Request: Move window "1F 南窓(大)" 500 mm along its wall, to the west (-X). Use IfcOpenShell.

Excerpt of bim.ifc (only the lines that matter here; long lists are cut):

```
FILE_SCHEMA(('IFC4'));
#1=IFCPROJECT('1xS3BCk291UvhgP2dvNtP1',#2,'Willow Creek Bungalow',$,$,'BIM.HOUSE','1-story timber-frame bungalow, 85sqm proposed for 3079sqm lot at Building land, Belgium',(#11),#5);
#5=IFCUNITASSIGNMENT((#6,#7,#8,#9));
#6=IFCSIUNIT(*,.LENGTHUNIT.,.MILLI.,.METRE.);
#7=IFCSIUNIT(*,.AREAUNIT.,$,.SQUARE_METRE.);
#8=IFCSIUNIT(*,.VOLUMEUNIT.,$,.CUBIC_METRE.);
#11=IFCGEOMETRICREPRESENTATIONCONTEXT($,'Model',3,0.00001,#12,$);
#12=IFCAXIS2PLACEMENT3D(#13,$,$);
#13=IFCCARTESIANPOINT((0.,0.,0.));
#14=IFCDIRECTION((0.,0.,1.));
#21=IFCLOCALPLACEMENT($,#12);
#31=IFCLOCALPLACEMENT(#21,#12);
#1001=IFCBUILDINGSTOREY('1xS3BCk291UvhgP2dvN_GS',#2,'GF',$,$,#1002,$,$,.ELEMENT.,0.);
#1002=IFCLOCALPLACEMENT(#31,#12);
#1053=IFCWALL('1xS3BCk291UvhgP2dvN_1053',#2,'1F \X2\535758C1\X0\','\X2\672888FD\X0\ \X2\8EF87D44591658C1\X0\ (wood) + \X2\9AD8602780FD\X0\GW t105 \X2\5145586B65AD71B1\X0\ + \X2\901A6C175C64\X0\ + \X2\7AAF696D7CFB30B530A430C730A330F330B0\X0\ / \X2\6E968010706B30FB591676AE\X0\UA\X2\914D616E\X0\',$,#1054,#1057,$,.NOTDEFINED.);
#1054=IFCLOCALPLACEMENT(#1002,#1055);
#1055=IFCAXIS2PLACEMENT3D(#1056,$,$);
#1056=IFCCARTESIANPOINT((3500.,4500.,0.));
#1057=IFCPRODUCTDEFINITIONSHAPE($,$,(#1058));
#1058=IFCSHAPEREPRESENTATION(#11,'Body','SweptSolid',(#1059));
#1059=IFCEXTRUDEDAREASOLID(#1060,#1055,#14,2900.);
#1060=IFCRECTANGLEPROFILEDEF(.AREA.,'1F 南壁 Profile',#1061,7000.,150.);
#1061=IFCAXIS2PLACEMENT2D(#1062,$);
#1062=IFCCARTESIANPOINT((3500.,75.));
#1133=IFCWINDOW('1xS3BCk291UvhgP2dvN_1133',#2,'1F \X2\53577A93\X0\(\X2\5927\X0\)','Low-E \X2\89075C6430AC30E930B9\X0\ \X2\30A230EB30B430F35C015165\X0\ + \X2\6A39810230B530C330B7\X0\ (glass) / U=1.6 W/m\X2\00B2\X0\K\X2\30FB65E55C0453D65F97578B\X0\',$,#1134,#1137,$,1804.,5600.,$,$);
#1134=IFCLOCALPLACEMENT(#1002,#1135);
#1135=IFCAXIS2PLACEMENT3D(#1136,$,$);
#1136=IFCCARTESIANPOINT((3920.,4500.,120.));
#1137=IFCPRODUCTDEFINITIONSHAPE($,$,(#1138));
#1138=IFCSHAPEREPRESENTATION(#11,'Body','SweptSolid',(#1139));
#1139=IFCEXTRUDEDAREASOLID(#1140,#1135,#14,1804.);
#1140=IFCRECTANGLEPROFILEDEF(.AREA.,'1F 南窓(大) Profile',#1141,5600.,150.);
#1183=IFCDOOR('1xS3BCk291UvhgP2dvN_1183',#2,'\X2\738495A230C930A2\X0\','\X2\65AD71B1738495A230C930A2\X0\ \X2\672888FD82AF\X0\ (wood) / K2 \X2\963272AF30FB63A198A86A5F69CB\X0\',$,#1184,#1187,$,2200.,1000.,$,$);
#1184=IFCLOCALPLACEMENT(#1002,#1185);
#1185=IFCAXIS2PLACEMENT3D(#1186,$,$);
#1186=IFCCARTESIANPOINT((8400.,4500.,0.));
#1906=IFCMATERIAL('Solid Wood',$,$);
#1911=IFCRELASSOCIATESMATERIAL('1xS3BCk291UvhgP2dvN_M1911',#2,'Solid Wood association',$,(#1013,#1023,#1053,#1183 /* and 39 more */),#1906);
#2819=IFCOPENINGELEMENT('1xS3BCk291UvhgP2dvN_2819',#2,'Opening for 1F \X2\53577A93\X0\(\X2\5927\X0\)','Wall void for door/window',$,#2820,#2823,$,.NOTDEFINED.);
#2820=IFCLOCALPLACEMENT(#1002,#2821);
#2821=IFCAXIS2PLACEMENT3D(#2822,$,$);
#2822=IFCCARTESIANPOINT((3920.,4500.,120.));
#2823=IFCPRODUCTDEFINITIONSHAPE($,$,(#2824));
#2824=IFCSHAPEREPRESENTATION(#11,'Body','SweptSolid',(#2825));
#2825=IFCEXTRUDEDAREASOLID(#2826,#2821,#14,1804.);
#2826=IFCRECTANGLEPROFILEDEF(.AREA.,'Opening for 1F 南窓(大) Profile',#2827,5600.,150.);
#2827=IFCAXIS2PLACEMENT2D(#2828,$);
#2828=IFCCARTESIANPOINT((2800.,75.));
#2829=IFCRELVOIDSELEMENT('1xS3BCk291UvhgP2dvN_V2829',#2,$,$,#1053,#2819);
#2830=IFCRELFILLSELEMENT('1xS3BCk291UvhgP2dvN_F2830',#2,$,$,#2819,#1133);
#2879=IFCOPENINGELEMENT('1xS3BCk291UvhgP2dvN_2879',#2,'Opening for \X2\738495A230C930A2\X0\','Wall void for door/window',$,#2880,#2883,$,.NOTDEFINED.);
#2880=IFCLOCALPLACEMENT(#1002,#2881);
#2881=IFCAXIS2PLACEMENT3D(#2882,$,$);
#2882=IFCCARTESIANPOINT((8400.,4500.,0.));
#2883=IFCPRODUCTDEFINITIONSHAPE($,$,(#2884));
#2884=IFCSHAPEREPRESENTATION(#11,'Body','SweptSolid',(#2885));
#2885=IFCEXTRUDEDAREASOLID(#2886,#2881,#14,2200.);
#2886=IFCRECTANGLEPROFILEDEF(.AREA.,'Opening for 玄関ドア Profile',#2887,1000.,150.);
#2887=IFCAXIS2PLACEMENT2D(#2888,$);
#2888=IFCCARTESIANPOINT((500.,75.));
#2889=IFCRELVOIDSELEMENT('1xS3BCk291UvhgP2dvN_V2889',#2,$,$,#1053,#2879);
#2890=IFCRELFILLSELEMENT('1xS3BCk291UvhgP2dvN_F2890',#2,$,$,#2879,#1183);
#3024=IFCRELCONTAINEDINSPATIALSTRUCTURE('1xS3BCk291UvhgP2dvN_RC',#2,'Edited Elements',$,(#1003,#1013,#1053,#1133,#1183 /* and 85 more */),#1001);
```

```python
import ifcopenshell
import ifcopenshell.api.geometry
import ifcopenshell.util.placement

model = ifcopenshell.open("bim.ifc")

window = model.by_guid("1xS3BCk291UvhgP2dvN_1133")
opening = window.FillsVoids[0].RelatingOpeningElement
wall = opening.VoidsElements[0].RelatingBuildingElement

wall_matrix = ifcopenshell.util.placement.get_local_placement(wall.ObjectPlacement)
shift = wall_matrix[:3, 0] * -500.0
before = ifcopenshell.util.placement.get_local_placement(window.ObjectPlacement)[:3, 3].copy()

# The window is not placed relative to its opening, so move both.
for product in (opening, window):
    matrix = ifcopenshell.util.placement.get_local_placement(product.ObjectPlacement)
    matrix[:3, 3] += shift
    ifcopenshell.api.geometry.edit_object_placement(model, product=product, matrix=matrix, is_si=False)

after = ifcopenshell.util.placement.get_local_placement(window.ObjectPlacement)[:3, 3]
print("window moved by", (after - before).round(3) + 0.0)

model.write("bim_rev.ifc")
```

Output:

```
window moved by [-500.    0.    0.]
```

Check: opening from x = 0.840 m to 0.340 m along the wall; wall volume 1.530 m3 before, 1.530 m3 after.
